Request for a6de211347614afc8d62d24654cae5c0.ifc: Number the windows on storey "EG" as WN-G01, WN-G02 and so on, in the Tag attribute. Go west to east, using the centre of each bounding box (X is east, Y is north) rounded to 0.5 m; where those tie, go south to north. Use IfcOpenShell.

First a look at what the model holds.

```python
import ifcopenshell
import ifcopenshell.util.element
import ifcopenshell.util.placement

model = ifcopenshell.open("a6de211347614afc8d62d24654cae5c0.ifc")
print(model.schema)
storey = next(s for s in model.by_type("IfcBuildingStorey") if s.Name == "EG")
windows = [e for e in ifcopenshell.util.element.get_decomposition(storey) if e.is_a("IfcWindow")]
for e in sorted(windows, key=lambda e: e.id()):
    origin = ifcopenshell.util.placement.get_local_placement(e.ObjectPlacement)[:3, 3]
    print(e.id(), e.Tag, e.Name, origin.round(2) + 0.0, sep=" | ")
```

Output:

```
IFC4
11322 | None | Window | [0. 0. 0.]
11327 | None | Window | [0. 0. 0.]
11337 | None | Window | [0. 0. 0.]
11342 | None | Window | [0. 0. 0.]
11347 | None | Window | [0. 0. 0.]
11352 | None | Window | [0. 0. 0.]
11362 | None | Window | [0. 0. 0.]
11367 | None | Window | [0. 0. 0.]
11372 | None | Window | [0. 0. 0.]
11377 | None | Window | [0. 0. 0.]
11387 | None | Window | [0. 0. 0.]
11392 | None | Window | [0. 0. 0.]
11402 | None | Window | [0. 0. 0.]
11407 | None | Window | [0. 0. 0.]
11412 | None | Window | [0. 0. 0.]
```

```python
import ifcopenshell
import ifcopenshell.geom
import ifcopenshell.util.element
import ifcopenshell.util.shape

model = ifcopenshell.open("a6de211347614afc8d62d24654cae5c0.ifc")
settings = ifcopenshell.geom.settings()
settings.set("use-world-coords", True)


def centre(element):
    shape = ifcopenshell.geom.create_shape(settings, element)
    return ifcopenshell.util.shape.get_bbox_centroid(shape.geometry)


storey = next(s for s in model.by_type("IfcBuildingStorey") if s.Name == "EG")
windows = [e for e in ifcopenshell.util.element.get_decomposition(storey) if e.is_a("IfcWindow")]

# Insertion points can sit at a corner or the storey origin, so sort by the geometry (in metres).
centres = {e: centre(e) for e in windows}
windows.sort(key=lambda e: (round(centres[e][0] / 0.5), centres[e][1]))

for i, e in enumerate(windows, start=1):
    number = f"WN-G{i:02d}"
    e.Tag = number
    print(e.id(), number)

model.write("a6de211347614afc8d62d24654cae5c0_updated.ifc")
```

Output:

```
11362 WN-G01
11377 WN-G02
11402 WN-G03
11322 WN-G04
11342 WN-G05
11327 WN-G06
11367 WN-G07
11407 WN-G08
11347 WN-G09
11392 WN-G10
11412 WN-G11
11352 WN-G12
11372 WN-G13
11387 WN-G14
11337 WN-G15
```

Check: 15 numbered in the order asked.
